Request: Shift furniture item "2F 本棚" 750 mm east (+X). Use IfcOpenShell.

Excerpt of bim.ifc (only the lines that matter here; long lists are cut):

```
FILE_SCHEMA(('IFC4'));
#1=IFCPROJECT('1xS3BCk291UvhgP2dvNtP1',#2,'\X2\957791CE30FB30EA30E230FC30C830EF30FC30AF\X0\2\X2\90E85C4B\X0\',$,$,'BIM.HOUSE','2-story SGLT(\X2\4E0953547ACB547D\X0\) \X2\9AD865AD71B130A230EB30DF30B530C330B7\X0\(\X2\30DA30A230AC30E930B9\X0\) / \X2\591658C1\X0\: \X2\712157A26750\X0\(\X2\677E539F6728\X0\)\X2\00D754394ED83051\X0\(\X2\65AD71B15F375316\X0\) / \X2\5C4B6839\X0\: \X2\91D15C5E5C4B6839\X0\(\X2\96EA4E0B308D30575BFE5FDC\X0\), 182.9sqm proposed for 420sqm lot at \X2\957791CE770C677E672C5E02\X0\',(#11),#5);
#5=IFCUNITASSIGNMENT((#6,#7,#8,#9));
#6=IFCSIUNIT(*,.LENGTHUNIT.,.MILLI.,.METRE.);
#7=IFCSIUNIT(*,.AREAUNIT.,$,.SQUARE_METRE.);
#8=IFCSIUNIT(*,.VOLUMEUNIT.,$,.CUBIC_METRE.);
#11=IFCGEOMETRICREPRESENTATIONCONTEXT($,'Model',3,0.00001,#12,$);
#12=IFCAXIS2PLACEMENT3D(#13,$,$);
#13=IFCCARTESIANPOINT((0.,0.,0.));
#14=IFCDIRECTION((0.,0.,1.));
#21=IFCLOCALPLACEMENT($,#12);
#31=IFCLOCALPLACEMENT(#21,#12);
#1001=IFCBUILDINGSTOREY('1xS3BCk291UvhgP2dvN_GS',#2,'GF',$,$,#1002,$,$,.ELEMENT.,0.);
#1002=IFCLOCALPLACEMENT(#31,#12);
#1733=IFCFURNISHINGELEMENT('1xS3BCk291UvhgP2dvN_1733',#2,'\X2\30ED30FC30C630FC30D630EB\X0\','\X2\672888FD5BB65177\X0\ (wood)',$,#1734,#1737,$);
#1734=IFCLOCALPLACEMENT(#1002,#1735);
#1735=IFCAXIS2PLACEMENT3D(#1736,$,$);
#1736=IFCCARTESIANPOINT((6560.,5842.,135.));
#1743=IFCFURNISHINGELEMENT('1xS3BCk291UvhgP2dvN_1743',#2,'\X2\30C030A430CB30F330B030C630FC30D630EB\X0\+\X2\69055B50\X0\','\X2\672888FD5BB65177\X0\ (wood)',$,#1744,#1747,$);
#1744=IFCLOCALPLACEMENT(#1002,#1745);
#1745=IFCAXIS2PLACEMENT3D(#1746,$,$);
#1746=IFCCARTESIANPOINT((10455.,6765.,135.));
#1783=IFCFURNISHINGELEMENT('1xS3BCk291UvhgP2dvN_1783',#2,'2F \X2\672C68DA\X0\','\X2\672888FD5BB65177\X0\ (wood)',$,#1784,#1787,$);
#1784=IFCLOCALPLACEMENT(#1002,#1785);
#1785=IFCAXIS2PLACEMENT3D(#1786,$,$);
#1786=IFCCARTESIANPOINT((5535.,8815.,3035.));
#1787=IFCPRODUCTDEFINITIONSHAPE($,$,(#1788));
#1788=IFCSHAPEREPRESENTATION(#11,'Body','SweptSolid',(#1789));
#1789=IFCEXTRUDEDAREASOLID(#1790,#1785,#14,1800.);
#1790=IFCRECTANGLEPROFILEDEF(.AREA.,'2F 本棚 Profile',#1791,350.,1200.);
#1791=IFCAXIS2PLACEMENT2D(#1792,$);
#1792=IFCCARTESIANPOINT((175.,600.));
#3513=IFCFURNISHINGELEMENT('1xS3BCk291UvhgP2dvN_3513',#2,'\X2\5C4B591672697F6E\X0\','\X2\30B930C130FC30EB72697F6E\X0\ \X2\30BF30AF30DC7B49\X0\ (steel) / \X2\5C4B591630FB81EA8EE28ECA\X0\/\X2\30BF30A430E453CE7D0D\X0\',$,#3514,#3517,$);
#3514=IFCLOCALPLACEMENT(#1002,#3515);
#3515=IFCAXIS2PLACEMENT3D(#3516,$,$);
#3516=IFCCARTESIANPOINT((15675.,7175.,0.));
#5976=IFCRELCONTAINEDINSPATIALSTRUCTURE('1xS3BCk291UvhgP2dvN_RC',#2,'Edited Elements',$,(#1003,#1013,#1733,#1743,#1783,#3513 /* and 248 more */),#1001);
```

```python
import ifcopenshell
import ifcopenshell.api.geometry
import ifcopenshell.util.placement
import ifcopenshell.util.unit

model = ifcopenshell.open("bim.ifc")
unit_scale = ifcopenshell.util.unit.calculate_unit_scale(model)

item = model.by_id(1783)
matrix = ifcopenshell.util.placement.get_local_placement(item.ObjectPlacement)
matrix[0, 3] += 0.75 / unit_scale
ifcopenshell.api.geometry.edit_object_placement(model, product=item, matrix=matrix, is_si=False)

print(ifcopenshell.util.placement.get_local_placement(item.ObjectPlacement).round(3) + 0.0)

model.write("bim_v2.ifc")
```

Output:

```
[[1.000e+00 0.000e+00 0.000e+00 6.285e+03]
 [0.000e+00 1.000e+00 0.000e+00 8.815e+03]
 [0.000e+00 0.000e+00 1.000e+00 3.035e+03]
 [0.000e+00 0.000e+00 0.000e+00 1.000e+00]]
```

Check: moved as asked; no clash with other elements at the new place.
